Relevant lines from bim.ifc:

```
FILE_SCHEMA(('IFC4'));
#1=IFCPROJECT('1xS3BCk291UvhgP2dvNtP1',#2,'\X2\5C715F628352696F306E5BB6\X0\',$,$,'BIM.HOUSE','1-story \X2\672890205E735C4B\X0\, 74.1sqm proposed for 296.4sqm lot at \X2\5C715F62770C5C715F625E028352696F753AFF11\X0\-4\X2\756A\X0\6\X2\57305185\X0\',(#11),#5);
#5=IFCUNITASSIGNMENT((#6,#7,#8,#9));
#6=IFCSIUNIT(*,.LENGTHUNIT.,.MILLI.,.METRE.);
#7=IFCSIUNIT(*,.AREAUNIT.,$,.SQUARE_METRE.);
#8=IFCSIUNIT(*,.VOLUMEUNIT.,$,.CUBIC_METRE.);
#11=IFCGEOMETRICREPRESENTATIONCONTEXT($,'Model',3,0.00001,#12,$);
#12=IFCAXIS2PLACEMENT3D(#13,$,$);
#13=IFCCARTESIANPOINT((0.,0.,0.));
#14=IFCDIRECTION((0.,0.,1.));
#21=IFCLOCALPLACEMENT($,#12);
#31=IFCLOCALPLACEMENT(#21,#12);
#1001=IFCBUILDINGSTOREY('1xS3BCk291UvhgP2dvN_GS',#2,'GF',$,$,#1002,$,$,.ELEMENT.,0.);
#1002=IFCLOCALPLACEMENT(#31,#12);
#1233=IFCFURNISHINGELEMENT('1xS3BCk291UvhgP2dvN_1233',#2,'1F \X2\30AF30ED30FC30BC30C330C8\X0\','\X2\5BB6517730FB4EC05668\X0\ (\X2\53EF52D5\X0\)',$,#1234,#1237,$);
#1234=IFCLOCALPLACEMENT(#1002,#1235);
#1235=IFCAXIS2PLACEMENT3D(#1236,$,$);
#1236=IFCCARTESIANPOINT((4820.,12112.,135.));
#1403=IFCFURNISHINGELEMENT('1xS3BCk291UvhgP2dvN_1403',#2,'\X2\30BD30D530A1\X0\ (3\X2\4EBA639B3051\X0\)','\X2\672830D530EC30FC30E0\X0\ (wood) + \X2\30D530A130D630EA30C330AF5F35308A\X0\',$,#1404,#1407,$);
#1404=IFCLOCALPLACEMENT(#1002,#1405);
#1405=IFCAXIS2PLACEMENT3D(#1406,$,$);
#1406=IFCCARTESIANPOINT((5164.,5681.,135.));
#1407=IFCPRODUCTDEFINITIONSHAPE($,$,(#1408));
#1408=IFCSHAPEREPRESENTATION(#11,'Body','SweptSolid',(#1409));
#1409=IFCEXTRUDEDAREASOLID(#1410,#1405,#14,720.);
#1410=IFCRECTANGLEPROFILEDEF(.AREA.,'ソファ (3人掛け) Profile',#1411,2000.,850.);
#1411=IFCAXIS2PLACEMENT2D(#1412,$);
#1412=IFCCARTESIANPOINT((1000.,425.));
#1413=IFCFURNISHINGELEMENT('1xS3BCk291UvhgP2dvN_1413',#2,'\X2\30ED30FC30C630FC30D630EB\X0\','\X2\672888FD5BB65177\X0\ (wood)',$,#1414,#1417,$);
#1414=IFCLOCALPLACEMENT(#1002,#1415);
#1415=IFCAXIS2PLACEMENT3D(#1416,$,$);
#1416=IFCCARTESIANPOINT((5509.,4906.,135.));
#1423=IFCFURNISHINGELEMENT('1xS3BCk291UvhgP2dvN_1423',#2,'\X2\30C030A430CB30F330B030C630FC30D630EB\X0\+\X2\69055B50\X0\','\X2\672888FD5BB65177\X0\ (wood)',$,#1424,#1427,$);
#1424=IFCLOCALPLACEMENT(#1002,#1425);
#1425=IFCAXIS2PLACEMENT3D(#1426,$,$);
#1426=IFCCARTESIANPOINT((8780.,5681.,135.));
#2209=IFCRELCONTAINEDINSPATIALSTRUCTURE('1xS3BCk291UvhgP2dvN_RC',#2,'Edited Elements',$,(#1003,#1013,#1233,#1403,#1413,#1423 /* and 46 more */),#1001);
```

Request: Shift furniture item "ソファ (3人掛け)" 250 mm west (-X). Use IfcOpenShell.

```python
import ifcopenshell
import ifcopenshell.api.geometry
import ifcopenshell.util.placement

model = ifcopenshell.open("bim.ifc")

item = model.by_guid("1xS3BCk291UvhgP2dvN_1403")
matrix = ifcopenshell.util.placement.get_local_placement(item.ObjectPlacement)
matrix[0, 3] -= 250.0
ifcopenshell.api.geometry.edit_object_placement(model, product=item, matrix=matrix, is_si=False)

print(ifcopenshell.util.placement.get_local_placement(item.ObjectPlacement).round(3) + 0.0)

model.write("bim-out.ifc")
```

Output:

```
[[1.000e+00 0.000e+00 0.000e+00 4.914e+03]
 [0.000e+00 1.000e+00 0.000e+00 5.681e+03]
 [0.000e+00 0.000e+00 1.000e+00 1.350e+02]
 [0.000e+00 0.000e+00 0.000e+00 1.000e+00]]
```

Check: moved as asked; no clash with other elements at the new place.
